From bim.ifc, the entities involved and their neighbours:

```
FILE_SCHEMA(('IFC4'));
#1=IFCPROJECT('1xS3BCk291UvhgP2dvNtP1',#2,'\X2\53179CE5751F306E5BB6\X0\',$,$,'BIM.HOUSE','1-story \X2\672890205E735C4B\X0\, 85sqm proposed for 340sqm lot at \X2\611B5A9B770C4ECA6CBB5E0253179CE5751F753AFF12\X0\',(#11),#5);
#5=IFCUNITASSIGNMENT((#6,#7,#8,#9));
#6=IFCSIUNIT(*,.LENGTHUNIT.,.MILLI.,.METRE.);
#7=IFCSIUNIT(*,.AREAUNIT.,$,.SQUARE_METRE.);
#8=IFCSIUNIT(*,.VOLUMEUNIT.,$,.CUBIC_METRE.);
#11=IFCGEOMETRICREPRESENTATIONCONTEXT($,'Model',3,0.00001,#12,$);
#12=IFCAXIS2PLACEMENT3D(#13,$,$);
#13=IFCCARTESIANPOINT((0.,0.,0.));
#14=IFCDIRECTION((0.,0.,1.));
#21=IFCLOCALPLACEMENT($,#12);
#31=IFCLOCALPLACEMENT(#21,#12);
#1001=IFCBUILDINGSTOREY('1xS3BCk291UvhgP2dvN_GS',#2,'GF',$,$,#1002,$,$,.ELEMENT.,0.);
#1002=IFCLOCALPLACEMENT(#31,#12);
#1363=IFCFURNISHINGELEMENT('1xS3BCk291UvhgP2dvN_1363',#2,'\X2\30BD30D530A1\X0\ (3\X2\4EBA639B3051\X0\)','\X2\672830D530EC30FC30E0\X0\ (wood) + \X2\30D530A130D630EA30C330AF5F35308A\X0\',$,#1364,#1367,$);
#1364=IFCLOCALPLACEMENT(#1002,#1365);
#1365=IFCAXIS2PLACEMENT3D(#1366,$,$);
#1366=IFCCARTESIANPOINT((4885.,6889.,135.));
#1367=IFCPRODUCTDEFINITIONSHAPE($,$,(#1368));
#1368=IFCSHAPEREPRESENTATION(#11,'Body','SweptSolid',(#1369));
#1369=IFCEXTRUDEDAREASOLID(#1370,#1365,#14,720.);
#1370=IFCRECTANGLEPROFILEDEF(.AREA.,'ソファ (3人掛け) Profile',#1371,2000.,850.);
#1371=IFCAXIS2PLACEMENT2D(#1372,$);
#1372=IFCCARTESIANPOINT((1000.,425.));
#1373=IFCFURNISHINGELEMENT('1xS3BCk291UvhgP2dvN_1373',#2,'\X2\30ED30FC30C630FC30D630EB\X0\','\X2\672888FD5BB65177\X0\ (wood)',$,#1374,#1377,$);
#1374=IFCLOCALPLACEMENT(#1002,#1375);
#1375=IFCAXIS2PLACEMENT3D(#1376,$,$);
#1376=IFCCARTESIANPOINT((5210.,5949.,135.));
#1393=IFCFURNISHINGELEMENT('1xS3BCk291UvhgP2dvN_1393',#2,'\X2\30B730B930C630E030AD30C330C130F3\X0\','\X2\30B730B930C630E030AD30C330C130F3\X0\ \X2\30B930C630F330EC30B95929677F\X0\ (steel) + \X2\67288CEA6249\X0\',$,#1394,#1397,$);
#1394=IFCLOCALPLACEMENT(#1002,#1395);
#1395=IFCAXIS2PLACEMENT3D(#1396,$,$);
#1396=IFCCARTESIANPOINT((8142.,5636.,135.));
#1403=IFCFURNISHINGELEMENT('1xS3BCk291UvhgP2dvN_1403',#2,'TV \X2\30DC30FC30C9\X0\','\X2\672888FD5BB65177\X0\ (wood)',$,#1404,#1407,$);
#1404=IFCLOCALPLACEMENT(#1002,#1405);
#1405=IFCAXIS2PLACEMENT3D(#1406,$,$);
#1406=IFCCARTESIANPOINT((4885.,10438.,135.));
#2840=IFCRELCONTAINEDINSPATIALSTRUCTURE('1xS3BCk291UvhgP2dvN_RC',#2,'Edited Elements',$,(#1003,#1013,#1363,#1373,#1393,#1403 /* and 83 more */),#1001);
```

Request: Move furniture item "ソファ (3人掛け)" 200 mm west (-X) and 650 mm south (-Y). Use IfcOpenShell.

```python
import ifcopenshell
import ifcopenshell.api.geometry
import ifcopenshell.util.placement

model = ifcopenshell.open("bim.ifc")

item = model.by_guid("1xS3BCk291UvhgP2dvN_1363")
matrix = ifcopenshell.util.placement.get_local_placement(item.ObjectPlacement)
matrix[0, 3] -= 200.0
matrix[1, 3] -= 650.0
ifcopenshell.api.geometry.edit_object_placement(model, product=item, matrix=matrix, is_si=False)

print(ifcopenshell.util.placement.get_local_placement(item.ObjectPlacement).round(3) + 0.0)

model.write("bim_rev.ifc")
```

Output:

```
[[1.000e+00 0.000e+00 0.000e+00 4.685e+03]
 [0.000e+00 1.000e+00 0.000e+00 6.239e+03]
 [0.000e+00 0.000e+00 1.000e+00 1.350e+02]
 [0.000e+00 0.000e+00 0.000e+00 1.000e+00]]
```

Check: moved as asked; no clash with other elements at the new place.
